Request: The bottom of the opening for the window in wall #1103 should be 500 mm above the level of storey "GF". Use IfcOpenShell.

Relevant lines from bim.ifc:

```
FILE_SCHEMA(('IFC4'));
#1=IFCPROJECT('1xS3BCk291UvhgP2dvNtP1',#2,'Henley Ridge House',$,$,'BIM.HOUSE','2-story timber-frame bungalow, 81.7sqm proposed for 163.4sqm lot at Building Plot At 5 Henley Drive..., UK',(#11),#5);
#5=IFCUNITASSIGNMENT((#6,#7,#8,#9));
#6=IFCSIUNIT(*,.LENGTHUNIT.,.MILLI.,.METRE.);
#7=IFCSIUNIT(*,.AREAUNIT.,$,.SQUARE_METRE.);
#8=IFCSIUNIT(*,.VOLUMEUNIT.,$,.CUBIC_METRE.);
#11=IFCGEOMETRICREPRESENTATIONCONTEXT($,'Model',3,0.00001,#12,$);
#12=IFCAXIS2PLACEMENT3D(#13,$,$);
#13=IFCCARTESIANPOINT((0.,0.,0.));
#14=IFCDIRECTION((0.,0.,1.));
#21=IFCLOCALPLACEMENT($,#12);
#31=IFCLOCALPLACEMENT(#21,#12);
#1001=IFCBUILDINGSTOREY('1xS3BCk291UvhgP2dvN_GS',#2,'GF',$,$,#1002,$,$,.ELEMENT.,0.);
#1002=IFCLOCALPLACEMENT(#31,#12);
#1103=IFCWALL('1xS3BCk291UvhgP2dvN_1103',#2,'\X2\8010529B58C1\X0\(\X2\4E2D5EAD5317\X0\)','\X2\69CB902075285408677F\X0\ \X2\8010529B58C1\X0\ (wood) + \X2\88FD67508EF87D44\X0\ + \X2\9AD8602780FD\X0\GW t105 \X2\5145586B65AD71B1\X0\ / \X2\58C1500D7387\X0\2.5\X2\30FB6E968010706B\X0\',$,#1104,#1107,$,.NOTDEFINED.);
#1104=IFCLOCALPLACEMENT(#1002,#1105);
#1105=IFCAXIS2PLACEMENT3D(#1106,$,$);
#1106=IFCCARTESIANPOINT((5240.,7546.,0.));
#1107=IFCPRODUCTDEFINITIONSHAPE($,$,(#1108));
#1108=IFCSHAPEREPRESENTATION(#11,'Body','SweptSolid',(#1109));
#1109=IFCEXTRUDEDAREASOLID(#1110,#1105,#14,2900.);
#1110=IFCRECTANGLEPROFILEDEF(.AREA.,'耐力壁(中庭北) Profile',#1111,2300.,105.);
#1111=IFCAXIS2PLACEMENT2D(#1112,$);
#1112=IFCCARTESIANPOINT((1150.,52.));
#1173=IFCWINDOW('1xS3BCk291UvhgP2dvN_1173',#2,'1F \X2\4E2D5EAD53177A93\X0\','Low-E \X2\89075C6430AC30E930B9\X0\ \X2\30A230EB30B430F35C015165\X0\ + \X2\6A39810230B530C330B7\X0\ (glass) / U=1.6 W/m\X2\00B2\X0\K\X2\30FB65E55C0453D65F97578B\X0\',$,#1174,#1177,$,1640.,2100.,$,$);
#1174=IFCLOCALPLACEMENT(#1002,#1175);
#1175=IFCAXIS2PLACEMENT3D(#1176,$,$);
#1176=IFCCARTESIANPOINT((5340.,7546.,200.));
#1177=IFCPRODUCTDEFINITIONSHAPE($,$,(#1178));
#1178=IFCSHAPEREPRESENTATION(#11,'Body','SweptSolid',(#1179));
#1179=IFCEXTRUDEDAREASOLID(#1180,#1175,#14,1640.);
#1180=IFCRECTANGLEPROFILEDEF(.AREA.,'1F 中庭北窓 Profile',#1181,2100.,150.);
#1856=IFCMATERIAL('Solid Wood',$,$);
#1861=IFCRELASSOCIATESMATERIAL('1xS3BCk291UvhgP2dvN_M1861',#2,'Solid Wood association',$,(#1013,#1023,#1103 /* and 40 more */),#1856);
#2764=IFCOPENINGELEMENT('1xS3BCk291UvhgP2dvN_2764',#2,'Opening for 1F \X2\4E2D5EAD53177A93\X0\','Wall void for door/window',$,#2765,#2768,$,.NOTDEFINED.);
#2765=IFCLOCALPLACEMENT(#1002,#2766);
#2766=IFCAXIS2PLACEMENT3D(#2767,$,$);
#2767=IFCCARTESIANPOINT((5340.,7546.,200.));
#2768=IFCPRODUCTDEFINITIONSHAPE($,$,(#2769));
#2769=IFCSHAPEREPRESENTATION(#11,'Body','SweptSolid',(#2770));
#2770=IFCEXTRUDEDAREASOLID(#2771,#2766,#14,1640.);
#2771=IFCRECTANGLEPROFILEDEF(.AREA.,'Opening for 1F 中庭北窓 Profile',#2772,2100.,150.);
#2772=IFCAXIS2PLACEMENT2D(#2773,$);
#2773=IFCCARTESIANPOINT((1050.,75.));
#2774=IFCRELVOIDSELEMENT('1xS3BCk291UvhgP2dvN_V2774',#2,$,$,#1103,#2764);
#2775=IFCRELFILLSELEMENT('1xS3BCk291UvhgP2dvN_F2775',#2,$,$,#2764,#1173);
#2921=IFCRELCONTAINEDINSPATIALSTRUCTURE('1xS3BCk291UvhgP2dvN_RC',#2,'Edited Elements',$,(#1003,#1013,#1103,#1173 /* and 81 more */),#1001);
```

```python
import numpy as np
import ifcopenshell
import ifcopenshell.api.geometry
import ifcopenshell.geom
import ifcopenshell.util.element
import ifcopenshell.util.placement
import ifcopenshell.util.shape
import ifcopenshell.util.unit

model = ifcopenshell.open("bim.ifc")
unit_scale = ifcopenshell.util.unit.calculate_unit_scale(model)

window = model.by_guid("1xS3BCk291UvhgP2dvN_1173")
opening = window.FillsVoids[0].RelatingOpeningElement
storey = ifcopenshell.util.element.get_container(window, ifc_class="IfcBuildingStorey")
level = ifcopenshell.util.placement.get_local_placement(storey.ObjectPlacement)[2, 3]

# The opening's origin need not be at the sill, so measure its lowest point.
shape = ifcopenshell.geom.create_shape(ifcopenshell.geom.settings(), opening)
bottom = ifcopenshell.util.shape.get_shape_bottom_elevation(shape, shape.geometry) / unit_scale
dz = level + 0.5 / unit_scale - bottom

shift = np.array([0.0, 0.0, dz])
# The window is not placed relative to its opening, so move both.
for product in (opening, window):
    matrix = ifcopenshell.util.placement.get_local_placement(product.ObjectPlacement)
    matrix[:3, 3] += shift
    ifcopenshell.api.geometry.edit_object_placement(model, product=product, matrix=matrix, is_si=False)

print(f"moved by {dz * unit_scale:+.3f} m")

model.write("bim-out.ifc")
```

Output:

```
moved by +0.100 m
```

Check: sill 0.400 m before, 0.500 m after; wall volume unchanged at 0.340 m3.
